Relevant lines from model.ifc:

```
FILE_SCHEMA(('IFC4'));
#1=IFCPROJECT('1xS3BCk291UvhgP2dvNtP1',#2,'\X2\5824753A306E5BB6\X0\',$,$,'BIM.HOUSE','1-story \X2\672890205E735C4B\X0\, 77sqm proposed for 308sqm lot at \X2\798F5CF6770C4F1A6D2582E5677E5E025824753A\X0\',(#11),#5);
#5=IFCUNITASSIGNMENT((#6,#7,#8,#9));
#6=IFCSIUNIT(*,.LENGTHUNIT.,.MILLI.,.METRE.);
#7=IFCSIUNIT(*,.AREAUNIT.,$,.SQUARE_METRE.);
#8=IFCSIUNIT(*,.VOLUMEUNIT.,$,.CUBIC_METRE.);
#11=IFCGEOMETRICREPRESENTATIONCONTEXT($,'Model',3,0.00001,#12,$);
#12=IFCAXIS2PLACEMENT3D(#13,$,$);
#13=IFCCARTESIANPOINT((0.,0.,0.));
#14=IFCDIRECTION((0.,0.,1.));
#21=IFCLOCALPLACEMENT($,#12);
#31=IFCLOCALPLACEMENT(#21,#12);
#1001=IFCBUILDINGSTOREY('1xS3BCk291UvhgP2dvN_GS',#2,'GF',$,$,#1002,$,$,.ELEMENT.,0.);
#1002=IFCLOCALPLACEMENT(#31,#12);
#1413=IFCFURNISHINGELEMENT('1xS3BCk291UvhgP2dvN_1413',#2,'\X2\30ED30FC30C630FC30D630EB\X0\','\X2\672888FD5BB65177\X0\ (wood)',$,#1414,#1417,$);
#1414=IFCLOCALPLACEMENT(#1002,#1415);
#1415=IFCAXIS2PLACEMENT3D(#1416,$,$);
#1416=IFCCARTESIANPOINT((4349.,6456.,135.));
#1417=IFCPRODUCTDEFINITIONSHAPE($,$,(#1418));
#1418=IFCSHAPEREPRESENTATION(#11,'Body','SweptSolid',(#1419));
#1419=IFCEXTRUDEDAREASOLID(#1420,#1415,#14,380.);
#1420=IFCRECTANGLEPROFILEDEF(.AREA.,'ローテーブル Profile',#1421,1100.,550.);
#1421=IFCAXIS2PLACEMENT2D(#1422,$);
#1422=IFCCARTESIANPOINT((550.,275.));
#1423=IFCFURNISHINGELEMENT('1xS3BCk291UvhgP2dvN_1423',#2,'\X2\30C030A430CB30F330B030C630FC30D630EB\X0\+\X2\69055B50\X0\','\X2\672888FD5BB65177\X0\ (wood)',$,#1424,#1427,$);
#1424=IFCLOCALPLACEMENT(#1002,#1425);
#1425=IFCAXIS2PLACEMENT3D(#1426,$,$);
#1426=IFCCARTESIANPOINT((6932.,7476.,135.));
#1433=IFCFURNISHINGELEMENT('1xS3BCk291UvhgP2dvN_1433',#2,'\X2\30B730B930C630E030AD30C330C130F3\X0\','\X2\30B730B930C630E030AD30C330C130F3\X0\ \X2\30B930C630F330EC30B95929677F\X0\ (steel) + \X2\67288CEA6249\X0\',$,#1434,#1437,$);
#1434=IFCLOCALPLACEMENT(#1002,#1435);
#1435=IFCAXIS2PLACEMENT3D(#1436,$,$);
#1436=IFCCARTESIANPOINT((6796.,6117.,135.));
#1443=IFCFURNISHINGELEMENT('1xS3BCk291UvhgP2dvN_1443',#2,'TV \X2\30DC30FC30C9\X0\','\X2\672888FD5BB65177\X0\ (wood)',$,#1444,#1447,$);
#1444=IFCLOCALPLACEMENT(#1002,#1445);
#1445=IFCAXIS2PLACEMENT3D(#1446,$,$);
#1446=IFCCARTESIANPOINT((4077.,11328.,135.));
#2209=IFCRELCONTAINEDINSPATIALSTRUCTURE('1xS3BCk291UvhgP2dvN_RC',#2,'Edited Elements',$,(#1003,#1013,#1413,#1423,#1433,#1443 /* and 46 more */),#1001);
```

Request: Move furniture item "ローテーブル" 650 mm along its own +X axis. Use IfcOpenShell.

```python
import ifcopenshell
import ifcopenshell.api.geometry
import ifcopenshell.util.placement

model = ifcopenshell.open("model.ifc")

item = model.by_id(1413)
matrix = ifcopenshell.util.placement.get_local_placement(item.ObjectPlacement)
matrix[:3, 3] += matrix[:3, 0] * 650.0
ifcopenshell.api.geometry.edit_object_placement(model, product=item, matrix=matrix, is_si=False)

print(ifcopenshell.util.placement.get_local_placement(item.ObjectPlacement).round(3) + 0.0)

model.write("model_rev.ifc")
```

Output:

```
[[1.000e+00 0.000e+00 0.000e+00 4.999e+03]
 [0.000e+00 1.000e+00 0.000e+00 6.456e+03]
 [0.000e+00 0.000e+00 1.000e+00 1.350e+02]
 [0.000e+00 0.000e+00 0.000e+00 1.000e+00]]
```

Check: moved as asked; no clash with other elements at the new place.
